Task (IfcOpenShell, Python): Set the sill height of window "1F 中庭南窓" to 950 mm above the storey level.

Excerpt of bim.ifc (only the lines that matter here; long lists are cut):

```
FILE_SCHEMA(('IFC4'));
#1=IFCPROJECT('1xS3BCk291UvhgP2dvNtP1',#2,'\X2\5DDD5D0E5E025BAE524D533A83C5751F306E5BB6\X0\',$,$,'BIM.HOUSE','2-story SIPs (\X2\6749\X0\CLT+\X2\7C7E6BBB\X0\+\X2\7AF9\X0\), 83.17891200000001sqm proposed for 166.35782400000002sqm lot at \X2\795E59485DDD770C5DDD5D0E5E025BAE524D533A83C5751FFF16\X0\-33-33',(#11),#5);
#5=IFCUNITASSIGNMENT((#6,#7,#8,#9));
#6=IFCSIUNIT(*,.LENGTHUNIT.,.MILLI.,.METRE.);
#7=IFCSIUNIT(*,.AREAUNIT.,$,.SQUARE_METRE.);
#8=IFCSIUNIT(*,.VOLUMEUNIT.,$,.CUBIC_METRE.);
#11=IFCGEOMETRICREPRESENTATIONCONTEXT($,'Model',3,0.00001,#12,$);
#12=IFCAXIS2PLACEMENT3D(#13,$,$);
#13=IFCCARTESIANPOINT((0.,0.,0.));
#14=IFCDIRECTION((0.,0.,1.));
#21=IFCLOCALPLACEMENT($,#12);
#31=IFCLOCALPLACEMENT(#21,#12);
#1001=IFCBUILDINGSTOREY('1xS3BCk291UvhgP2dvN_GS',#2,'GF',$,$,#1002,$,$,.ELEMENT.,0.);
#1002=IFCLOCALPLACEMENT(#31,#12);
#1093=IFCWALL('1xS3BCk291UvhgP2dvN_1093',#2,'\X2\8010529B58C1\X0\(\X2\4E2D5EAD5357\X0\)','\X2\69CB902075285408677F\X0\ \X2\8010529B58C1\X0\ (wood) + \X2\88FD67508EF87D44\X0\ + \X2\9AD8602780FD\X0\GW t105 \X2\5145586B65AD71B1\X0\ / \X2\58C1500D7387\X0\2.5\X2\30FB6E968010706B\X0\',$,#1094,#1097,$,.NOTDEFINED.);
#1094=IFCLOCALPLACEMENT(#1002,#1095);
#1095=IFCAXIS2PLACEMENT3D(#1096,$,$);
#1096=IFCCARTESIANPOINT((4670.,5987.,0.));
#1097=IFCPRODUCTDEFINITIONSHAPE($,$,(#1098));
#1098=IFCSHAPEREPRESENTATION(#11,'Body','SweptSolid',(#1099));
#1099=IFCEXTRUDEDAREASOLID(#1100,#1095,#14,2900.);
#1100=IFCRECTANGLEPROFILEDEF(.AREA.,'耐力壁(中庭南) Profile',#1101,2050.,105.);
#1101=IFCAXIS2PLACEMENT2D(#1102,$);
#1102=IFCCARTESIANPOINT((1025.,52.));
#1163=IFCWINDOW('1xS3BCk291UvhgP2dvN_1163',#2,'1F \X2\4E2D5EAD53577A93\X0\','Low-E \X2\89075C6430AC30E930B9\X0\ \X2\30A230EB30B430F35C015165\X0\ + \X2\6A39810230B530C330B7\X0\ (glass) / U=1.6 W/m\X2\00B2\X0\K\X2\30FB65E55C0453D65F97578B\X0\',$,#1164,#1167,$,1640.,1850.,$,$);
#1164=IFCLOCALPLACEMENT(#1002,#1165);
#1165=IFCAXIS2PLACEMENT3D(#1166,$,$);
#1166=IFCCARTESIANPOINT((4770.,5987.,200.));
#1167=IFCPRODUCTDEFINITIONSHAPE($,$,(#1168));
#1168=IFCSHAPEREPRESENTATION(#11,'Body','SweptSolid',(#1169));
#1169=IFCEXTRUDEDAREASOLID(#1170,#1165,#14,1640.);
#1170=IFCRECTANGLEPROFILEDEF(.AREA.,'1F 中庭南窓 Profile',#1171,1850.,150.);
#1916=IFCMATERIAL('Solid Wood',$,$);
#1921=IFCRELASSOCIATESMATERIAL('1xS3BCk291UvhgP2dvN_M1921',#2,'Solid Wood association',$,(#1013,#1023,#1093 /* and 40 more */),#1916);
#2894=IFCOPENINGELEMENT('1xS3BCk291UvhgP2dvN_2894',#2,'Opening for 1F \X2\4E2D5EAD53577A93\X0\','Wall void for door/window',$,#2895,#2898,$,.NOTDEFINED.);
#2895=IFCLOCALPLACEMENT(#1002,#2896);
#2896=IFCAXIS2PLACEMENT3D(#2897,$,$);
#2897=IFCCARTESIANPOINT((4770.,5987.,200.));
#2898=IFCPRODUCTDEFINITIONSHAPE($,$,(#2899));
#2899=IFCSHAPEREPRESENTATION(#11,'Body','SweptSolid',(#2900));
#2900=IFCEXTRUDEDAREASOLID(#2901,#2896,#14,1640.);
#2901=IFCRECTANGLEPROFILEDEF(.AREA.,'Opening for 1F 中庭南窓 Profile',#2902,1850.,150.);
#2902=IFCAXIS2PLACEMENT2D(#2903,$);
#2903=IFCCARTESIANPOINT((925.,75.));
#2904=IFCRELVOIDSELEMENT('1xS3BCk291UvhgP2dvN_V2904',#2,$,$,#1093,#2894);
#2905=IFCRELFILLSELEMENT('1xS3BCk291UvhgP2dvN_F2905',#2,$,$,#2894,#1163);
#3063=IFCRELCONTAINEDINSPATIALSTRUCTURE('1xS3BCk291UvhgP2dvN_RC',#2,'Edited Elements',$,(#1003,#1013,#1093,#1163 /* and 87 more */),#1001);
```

```python
import numpy as np
import ifcopenshell
import ifcopenshell.api.geometry
import ifcopenshell.geom
import ifcopenshell.util.element
import ifcopenshell.util.placement
import ifcopenshell.util.shape
import ifcopenshell.util.unit

model = ifcopenshell.open("bim.ifc")
unit_scale = ifcopenshell.util.unit.calculate_unit_scale(model)

window = model.by_guid("1xS3BCk291UvhgP2dvN_1163")
opening = window.FillsVoids[0].RelatingOpeningElement
storey = ifcopenshell.util.element.get_container(window, ifc_class="IfcBuildingStorey")
level = ifcopenshell.util.placement.get_local_placement(storey.ObjectPlacement)[2, 3]

# The opening's origin need not be at the sill, so measure its lowest point.
shape = ifcopenshell.geom.create_shape(ifcopenshell.geom.settings(), opening)
bottom = ifcopenshell.util.shape.get_shape_bottom_elevation(shape, shape.geometry) / unit_scale
dz = level + 0.95 / unit_scale - bottom

shift = np.array([0.0, 0.0, dz])
# The window is not placed relative to its opening, so move both.
for product in (opening, window):
    matrix = ifcopenshell.util.placement.get_local_placement(product.ObjectPlacement)
    matrix[:3, 3] += shift
    ifcopenshell.api.geometry.edit_object_placement(model, product=product, matrix=matrix, is_si=False)

print(f"moved by {dz * unit_scale:+.3f} m")

model.write("bim_v2.ifc")
```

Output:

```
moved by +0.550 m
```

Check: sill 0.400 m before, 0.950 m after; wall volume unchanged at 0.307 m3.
